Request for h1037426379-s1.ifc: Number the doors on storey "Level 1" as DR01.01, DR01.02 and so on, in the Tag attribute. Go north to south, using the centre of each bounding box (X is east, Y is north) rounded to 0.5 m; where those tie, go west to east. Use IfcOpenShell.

First a look at what the model holds.

```python
import ifcopenshell
import ifcopenshell.util.element
import ifcopenshell.util.placement

model = ifcopenshell.open("h1037426379-s1.ifc")
print(model.schema)
storey = next(s for s in model.by_type("IfcBuildingStorey") if s.Name == "Level 1")
doors = [e for e in ifcopenshell.util.element.get_decomposition(storey) if e.is_a("IfcDoor")]
for e in sorted(doors, key=lambda e: e.id()):
    origin = ifcopenshell.util.placement.get_local_placement(e.ObjectPlacement)[:3, 3]
    print(e.id(), e.Tag, e.Name, origin.round(2) + 0.0, sep=" | ")
```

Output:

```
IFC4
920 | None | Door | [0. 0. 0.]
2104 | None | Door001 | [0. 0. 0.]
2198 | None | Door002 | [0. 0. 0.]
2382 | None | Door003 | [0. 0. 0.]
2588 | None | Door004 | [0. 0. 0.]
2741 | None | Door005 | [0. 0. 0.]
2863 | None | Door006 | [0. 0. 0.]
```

```python
import ifcopenshell
import ifcopenshell.geom
import ifcopenshell.util.element
import ifcopenshell.util.shape

model = ifcopenshell.open("h1037426379-s1.ifc")
settings = ifcopenshell.geom.settings()
settings.set("use-world-coords", True)


def centre(element):
    shape = ifcopenshell.geom.create_shape(settings, element)
    return ifcopenshell.util.shape.get_bbox_centroid(shape.geometry)


storey = next(s for s in model.by_type("IfcBuildingStorey") if s.Name == "Level 1")
doors = [e for e in ifcopenshell.util.element.get_decomposition(storey) if e.is_a("IfcDoor")]

# Insertion points can sit at a corner or the storey origin, so sort by the geometry (in metres).
centres = {e: centre(e) for e in doors}
doors.sort(key=lambda e: (-round(centres[e][1] / 0.5), centres[e][0]))

for i, e in enumerate(doors, start=1):
    number = f"DR01.{i:02d}"
    e.Tag = number
    print(e.id(), number)

model.write("h1037426379-s1_v2.ifc")
```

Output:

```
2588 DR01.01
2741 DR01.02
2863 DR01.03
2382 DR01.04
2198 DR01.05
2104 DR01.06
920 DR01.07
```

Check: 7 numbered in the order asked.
